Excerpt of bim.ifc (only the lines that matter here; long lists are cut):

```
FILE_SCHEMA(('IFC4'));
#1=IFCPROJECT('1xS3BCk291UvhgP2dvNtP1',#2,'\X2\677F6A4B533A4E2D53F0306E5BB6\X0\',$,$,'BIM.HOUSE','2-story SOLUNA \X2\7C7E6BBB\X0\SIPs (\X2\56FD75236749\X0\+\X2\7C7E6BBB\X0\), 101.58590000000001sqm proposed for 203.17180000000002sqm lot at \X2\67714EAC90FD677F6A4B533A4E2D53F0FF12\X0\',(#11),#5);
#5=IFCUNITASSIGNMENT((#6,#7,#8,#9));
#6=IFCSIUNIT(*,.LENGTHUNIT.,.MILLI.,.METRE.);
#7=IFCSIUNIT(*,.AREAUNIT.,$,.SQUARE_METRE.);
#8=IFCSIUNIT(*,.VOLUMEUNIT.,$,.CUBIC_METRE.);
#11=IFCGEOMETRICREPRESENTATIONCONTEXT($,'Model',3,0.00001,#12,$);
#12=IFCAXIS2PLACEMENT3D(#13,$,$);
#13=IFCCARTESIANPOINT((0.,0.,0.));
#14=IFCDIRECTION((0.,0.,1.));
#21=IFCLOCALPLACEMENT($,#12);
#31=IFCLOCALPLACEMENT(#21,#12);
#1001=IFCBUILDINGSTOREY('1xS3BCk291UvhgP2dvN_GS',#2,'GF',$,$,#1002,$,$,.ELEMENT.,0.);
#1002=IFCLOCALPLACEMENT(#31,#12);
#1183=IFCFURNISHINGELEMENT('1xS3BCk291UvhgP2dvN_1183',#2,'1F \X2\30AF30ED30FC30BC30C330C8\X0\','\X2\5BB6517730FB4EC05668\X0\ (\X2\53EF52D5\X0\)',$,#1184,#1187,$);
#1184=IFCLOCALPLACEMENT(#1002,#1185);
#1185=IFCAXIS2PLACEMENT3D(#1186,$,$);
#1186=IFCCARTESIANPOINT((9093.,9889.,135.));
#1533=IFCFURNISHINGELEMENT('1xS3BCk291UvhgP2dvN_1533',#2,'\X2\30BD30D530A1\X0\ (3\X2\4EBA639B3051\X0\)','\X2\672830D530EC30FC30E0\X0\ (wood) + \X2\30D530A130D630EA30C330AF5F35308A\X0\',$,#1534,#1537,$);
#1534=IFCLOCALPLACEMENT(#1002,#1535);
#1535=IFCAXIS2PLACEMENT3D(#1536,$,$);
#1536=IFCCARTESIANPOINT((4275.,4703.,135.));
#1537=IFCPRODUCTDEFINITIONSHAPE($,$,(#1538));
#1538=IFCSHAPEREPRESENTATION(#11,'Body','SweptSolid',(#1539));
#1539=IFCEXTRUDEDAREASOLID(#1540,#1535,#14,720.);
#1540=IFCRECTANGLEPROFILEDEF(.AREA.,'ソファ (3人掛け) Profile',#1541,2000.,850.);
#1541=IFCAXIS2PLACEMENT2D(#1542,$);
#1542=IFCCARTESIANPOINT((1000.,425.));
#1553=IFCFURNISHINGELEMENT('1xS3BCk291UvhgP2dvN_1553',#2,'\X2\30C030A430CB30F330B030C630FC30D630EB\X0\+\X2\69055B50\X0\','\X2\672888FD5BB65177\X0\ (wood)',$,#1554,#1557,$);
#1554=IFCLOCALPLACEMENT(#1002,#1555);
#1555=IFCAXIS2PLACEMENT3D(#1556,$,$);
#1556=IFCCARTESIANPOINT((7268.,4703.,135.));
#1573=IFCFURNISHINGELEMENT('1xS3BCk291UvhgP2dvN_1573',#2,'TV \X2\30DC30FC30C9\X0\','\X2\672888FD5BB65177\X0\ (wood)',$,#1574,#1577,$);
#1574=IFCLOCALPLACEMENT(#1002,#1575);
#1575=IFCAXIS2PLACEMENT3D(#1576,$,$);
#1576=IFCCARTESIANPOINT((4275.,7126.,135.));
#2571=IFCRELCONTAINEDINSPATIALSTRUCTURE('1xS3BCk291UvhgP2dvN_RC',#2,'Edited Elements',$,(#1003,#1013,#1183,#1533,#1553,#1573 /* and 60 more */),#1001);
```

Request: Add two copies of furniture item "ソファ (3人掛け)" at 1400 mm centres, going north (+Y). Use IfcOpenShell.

```python
import numpy as np
import ifcopenshell
import ifcopenshell.api.geometry
import ifcopenshell.api.root
import ifcopenshell.util.element
import ifcopenshell.util.placement
import ifcopenshell.util.unit

model = ifcopenshell.open("bim.ifc")
unit_scale = ifcopenshell.util.unit.calculate_unit_scale(model)


def reuse_history(source, copy):
    """copy_class also copies each property set's owner history, people and application; keep the originals."""
    for rel in copy.IsDefinedBy:
        if rel.is_a("IfcRelDefinesByProperties") and (history := rel.RelatingPropertyDefinition.OwnerHistory):
            rel.RelatingPropertyDefinition.OwnerHistory = source.OwnerHistory
            ifcopenshell.util.element.remove_deep2(model, history)


source = model.by_id(1533)
base = ifcopenshell.util.placement.get_local_placement(source.ObjectPlacement)
step = np.array([0.0, 1.0, 0.0]) * 1.4 / unit_scale

for i in range(1, 3):
    copy = ifcopenshell.api.root.copy_class(model, product=source)
    copy.Representation = ifcopenshell.util.element.copy_deep(
        model, source.Representation, exclude=["IfcGeometricRepresentationContext", "IfcRepresentationMap"]
    )
    reuse_history(source, copy)
    matrix = base.copy()
    matrix[:3, 3] += i * step
    print("added at", matrix[:3, 3].round(3) + 0.0)
    ifcopenshell.api.geometry.edit_object_placement(model, product=copy, matrix=matrix, is_si=False)

model.write("bim_edited.ifc")
```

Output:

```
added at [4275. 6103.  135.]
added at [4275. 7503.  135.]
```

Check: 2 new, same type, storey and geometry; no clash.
